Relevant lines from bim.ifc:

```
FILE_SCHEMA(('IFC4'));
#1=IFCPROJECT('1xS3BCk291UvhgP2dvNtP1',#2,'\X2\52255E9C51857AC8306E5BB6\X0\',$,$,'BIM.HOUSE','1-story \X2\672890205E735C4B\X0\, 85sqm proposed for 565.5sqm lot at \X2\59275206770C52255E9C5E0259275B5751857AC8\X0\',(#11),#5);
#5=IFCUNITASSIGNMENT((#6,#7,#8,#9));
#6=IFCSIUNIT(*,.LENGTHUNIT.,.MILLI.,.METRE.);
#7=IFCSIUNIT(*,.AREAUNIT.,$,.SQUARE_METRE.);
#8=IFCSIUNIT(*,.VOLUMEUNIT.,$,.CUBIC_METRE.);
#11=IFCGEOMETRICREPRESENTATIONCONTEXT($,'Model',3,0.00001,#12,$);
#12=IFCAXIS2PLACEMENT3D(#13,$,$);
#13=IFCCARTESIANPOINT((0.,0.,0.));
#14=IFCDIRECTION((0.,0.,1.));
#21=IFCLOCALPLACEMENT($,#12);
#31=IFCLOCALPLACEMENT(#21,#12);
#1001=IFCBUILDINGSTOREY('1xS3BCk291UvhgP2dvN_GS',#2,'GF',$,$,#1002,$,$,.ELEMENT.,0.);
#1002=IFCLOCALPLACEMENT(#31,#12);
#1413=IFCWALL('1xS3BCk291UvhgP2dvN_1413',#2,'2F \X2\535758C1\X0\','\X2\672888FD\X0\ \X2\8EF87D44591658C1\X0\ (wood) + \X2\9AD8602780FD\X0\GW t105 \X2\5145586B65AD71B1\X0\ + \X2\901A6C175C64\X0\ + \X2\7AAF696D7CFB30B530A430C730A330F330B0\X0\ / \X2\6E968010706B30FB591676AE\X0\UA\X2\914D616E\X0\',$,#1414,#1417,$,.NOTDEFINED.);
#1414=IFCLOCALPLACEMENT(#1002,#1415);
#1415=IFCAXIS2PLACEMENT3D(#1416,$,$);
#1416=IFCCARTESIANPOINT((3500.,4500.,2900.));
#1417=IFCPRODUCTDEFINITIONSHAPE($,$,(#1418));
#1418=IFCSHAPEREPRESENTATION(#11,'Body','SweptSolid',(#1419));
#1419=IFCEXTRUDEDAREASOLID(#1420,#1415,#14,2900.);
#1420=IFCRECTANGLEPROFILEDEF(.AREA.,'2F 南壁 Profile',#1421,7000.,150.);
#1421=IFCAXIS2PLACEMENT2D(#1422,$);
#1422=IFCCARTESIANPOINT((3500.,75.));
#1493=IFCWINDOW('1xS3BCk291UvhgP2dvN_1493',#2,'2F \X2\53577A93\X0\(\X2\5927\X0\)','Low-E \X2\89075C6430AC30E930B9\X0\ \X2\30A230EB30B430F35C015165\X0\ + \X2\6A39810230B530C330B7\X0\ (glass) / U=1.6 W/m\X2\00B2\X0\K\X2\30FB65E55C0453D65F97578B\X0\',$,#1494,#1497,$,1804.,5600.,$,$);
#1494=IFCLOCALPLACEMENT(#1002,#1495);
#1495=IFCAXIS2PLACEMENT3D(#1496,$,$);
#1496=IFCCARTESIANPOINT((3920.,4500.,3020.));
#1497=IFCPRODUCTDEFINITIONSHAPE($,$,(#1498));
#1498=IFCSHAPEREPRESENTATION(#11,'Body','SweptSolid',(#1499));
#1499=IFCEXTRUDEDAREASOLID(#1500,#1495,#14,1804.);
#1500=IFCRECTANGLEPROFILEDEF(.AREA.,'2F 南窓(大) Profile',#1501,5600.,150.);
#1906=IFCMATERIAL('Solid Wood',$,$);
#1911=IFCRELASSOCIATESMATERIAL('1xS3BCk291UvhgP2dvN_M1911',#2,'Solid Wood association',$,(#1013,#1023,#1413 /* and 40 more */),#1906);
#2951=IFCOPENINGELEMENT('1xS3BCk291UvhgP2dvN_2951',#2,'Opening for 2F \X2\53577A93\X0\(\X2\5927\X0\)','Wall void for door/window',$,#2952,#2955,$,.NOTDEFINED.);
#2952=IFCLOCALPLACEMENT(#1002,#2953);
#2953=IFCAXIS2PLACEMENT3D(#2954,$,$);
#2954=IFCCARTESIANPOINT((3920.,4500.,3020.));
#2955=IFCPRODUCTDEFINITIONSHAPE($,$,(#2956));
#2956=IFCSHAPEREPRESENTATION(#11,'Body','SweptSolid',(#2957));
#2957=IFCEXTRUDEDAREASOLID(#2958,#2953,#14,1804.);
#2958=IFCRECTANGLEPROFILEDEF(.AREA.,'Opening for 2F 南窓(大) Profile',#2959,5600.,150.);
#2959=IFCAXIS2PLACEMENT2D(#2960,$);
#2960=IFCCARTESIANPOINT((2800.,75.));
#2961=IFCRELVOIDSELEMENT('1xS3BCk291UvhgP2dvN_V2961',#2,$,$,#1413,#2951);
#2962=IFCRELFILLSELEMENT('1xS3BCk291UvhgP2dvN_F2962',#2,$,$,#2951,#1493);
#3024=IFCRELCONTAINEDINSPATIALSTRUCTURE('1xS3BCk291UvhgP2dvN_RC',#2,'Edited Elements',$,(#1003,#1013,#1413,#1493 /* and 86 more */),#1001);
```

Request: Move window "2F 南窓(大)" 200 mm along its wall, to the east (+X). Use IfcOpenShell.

```python
import ifcopenshell
import ifcopenshell.api.geometry
import ifcopenshell.util.placement

model = ifcopenshell.open("bim.ifc")

window = model.by_guid("1xS3BCk291UvhgP2dvN_1493")
opening = window.FillsVoids[0].RelatingOpeningElement
wall = opening.VoidsElements[0].RelatingBuildingElement

wall_matrix = ifcopenshell.util.placement.get_local_placement(wall.ObjectPlacement)
shift = wall_matrix[:3, 0] * 200.0
before = ifcopenshell.util.placement.get_local_placement(window.ObjectPlacement)[:3, 3].copy()

# The window is not placed relative to its opening, so move both.
for product in (opening, window):
    matrix = ifcopenshell.util.placement.get_local_placement(product.ObjectPlacement)
    matrix[:3, 3] += shift
    ifcopenshell.api.geometry.edit_object_placement(model, product=product, matrix=matrix, is_si=False)

after = ifcopenshell.util.placement.get_local_placement(window.ObjectPlacement)[:3, 3]
print("window moved by", (after - before).round(3) + 0.0)

model.write("bim-out.ifc")
```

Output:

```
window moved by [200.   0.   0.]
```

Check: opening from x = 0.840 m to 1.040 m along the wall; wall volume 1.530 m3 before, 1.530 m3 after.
